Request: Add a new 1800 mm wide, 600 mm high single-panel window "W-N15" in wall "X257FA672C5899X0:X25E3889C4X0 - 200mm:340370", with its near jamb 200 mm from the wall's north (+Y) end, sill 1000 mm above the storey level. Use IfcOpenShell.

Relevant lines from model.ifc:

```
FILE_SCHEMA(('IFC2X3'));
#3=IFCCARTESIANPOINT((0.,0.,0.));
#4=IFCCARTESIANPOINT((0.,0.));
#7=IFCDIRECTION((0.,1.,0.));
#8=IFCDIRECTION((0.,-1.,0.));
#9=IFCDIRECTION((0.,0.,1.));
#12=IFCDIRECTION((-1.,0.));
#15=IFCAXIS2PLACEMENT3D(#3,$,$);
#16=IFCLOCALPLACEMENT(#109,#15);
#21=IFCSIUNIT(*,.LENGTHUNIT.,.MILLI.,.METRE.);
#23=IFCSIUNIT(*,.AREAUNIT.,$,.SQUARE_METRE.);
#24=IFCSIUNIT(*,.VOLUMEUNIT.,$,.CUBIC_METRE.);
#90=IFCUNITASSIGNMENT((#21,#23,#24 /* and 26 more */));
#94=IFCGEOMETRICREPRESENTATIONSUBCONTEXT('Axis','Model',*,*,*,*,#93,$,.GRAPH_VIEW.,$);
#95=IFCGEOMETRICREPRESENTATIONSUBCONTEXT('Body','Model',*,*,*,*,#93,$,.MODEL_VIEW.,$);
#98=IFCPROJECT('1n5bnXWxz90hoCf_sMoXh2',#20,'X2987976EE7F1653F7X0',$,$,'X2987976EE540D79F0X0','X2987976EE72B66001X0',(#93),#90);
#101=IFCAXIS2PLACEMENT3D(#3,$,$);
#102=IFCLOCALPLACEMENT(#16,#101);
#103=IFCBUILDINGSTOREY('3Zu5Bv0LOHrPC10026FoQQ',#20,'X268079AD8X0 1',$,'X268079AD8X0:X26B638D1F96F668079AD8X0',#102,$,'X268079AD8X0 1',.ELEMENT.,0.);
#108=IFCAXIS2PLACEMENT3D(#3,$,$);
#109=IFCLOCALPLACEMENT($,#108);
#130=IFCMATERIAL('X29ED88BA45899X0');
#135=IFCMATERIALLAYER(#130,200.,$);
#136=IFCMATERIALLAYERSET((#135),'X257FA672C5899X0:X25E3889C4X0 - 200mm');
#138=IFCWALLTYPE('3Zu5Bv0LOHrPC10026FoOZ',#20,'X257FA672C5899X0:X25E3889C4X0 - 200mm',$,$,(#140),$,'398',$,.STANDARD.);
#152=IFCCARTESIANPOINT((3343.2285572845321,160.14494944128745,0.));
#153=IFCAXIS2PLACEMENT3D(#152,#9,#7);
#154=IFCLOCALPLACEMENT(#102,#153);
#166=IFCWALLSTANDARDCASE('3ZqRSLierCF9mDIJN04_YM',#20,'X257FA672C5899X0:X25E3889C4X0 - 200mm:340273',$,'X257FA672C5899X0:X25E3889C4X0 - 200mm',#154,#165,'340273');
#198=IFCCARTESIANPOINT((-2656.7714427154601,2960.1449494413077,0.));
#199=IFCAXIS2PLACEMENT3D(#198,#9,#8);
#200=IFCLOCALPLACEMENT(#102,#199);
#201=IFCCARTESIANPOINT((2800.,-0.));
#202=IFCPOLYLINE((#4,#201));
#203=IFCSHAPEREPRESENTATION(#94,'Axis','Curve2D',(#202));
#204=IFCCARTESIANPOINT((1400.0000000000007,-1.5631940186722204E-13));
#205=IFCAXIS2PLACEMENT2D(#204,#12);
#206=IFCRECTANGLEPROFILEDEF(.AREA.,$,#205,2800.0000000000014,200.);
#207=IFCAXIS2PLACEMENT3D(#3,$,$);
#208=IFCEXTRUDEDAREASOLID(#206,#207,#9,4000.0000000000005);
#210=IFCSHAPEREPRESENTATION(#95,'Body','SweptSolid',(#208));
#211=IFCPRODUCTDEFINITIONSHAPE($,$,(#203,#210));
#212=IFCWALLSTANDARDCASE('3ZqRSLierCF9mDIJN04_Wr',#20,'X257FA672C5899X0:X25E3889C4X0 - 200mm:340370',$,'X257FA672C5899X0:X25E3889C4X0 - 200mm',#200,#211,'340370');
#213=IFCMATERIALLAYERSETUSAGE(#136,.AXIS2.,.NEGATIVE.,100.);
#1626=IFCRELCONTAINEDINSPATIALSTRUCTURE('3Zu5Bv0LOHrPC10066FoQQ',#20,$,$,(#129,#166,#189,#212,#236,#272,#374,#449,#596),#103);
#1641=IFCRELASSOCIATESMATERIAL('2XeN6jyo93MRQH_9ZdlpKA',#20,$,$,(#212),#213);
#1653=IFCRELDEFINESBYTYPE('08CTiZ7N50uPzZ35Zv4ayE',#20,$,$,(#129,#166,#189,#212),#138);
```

```python
import numpy as np
import ifcopenshell
import ifcopenshell.api.feature
import ifcopenshell.api.geometry
import ifcopenshell.api.root
import ifcopenshell.api.spatial
import ifcopenshell.api.type
import ifcopenshell.geom
import ifcopenshell.util.element
import ifcopenshell.util.placement
import ifcopenshell.util.representation
import ifcopenshell.util.shape
import ifcopenshell.util.unit

model = ifcopenshell.open("model.ifc")
unit_scale = ifcopenshell.util.unit.calculate_unit_scale(model)
settings = ifcopenshell.geom.settings()


def volume(element):
    """Net volume in cubic metres, openings subtracted."""
    shape = ifcopenshell.geom.create_shape(settings, element)
    return ifcopenshell.util.shape.get_volume(shape.geometry)


wall = model.by_id(212)
storey = ifcopenshell.util.element.get_container(wall, ifc_class="IfcBuildingStorey")
context = ifcopenshell.util.representation.get_context(model, "Model", "Body", "MODEL_VIEW")
before = volume(wall)

width, height, from_end, sill = 1.8, 0.6, 0.2, 1  # metres

# The wall runs along its own X axis, and the end named is its -X end.
wall_shape = ifcopenshell.geom.create_shape(settings, wall)
x, y, z = ifcopenshell.util.shape.get_vertices(wall_shape.geometry).T
start = x.min() + from_end
face, thickness = float(y.min()), float(y.max() - y.min())
wall_matrix = ifcopenshell.util.placement.get_local_placement(wall.ObjectPlacement)
level = ifcopenshell.util.placement.get_local_placement(storey.ObjectPlacement)[2, 3]


def in_wall(x, y):
    """Placement at x, y metres in the wall's axes, at sill height."""
    matrix = wall_matrix.copy()
    matrix[:, 3] = wall_matrix @ np.array([x / unit_scale, y / unit_scale, 0.0, 1.0])
    matrix[2, 3] = level + sill / unit_scale
    return matrix


# Opening: a box that overshoots both wall faces by 50 mm.
opening = ifcopenshell.api.root.create_entity(model, ifc_class="IfcOpeningElement")
box = ifcopenshell.api.geometry.add_wall_representation(
    model, context=context, length=width, height=height, thickness=thickness + 0.1
)
ifcopenshell.api.geometry.assign_representation(model, product=opening, representation=box)
ifcopenshell.api.geometry.edit_object_placement(model, product=opening, matrix=in_wall(start, face - 0.05), is_si=False)
ifcopenshell.api.feature.add_feature(model, feature=opening, element=wall)

window = ifcopenshell.api.root.create_entity(model, ifc_class="IfcWindow", name="W-N15")
window.OverallWidth, window.OverallHeight = width / unit_scale, height / unit_scale
body = ifcopenshell.api.geometry.add_window_representation(
    model,
    context=context,
    overall_width=window.OverallWidth,
    overall_height=window.OverallHeight,
    partition_type="SINGLE_PANEL",
)
ifcopenshell.api.geometry.assign_representation(model, product=window, representation=body)
ifcopenshell.api.spatial.assign_container(model, products=[window], relating_structure=storey)
fills = ifcopenshell.api.feature.add_filling(model, opening=opening, element=window)
fills.OwnerHistory = window.OwnerHistory  # required in IFC2X3

# IFC2X3 keeps the operation on the window style.
style = ifcopenshell.api.root.create_entity(model, ifc_class="IfcWindowStyle", name="W-N15")
style.OperationType, style.ConstructionType = "SINGLE_PANEL", "NOTDEFINED"
style.ParameterTakesPrecedence = style.Sizeable = False
ifcopenshell.api.type.assign_type(model, related_objects=[window], relating_type=style)

# Centre the window in the wall's thickness.
ifcopenshell.api.geometry.edit_object_placement(model, product=window, matrix=in_wall(start, face), is_si=False)
window_shape = ifcopenshell.geom.create_shape(settings, window)
depth = ifcopenshell.util.shape.get_vertices(window_shape.geometry)[:, 1]
offset = face + thickness / 2 - (depth.min() + depth.max()) / 2
ifcopenshell.api.geometry.edit_object_placement(model, product=window, matrix=in_wall(start, offset), is_si=False)

after = volume(wall)

print(f"wall volume {before:.3f} -> {after:.3f} m3")

model.write("model_rev.ifc")
```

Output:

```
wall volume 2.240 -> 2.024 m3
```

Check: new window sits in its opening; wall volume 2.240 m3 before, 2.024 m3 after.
